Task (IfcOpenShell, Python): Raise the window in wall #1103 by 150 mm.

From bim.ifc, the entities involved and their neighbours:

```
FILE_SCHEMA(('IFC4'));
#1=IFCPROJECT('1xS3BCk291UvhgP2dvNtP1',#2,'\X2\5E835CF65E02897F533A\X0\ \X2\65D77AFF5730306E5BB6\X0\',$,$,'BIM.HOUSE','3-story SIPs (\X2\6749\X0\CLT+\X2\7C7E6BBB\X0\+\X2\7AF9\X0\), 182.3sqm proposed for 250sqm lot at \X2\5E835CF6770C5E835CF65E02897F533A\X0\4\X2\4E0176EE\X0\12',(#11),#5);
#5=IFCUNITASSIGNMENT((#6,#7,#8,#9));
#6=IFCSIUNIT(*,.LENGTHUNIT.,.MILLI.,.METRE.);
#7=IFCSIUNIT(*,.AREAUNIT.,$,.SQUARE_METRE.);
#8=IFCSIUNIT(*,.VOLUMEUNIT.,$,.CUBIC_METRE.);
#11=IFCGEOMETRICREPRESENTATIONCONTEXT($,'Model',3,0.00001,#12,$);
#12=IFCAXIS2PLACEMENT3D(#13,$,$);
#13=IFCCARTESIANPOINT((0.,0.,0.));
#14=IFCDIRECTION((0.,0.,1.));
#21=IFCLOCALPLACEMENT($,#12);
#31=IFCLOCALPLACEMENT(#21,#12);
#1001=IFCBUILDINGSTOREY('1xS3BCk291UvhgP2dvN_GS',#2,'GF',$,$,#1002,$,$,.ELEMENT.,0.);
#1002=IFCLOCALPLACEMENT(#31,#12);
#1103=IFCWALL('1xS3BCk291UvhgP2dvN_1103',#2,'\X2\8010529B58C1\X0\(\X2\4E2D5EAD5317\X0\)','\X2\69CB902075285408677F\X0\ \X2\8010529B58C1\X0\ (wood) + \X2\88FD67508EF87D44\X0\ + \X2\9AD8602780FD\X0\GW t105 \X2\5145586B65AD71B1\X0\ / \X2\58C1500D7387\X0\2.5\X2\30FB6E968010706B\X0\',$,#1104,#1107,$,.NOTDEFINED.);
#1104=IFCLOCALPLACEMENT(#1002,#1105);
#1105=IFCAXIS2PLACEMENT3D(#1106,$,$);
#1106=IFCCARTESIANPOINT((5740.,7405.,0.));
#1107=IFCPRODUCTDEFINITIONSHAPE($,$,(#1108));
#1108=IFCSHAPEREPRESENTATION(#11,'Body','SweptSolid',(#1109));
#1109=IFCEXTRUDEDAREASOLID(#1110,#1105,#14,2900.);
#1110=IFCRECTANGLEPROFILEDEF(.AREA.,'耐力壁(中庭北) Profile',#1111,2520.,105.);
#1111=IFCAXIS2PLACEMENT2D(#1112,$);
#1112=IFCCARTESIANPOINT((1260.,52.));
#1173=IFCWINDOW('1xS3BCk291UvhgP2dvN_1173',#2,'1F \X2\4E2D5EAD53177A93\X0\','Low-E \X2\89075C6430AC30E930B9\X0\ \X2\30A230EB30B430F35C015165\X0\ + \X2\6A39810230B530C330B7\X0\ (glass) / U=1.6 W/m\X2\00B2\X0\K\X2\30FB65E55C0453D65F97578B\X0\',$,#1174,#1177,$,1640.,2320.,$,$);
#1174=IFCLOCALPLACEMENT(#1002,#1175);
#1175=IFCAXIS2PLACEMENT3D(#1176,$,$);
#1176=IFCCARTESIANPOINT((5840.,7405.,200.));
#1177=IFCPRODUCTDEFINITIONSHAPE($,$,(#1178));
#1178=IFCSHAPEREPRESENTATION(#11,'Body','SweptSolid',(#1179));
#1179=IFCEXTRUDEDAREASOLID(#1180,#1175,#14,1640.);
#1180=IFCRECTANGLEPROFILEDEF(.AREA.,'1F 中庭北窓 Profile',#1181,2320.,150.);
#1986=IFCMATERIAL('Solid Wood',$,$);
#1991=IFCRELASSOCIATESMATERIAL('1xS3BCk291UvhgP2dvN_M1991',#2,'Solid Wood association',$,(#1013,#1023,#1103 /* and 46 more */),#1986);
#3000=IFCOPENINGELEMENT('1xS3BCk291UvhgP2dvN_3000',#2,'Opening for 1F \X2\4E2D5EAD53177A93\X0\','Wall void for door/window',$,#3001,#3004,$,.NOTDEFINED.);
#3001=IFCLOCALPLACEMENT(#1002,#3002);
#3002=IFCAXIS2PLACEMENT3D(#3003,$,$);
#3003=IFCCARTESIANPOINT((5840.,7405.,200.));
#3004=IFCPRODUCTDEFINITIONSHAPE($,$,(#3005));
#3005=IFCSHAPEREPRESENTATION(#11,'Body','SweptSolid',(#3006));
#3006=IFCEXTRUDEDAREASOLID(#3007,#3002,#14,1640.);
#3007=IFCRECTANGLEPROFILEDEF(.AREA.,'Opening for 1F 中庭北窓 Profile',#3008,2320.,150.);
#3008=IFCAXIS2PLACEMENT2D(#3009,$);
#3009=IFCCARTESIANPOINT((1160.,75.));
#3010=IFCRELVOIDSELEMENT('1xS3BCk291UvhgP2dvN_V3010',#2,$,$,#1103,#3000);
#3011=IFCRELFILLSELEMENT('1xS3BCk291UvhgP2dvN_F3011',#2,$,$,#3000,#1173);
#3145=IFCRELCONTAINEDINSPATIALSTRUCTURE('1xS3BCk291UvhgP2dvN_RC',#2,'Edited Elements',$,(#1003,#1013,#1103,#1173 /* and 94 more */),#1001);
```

```python
import numpy as np
import ifcopenshell
import ifcopenshell.api.geometry
import ifcopenshell.util.placement
import ifcopenshell.util.unit

model = ifcopenshell.open("bim.ifc")
unit_scale = ifcopenshell.util.unit.calculate_unit_scale(model)

window = model.by_guid("1xS3BCk291UvhgP2dvN_1173")
opening = window.FillsVoids[0].RelatingOpeningElement
dz = 0.15 / unit_scale

shift = np.array([0.0, 0.0, dz])
# The window is not placed relative to its opening, so move both.
for product in (opening, window):
    matrix = ifcopenshell.util.placement.get_local_placement(product.ObjectPlacement)
    matrix[:3, 3] += shift
    ifcopenshell.api.geometry.edit_object_placement(model, product=product, matrix=matrix, is_si=False)

print(f"moved by {dz * unit_scale:+.3f} m")

model.write("bim-out.ifc")
```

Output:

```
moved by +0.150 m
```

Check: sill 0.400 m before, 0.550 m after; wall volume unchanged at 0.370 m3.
